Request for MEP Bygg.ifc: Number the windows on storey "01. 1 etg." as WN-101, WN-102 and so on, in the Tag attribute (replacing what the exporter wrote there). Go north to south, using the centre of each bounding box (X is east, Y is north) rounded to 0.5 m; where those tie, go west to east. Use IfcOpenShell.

First a look at what the model holds.

```python
import ifcopenshell
import ifcopenshell.util.element
import ifcopenshell.util.placement

model = ifcopenshell.open("MEP Bygg.ifc")
print(model.schema)
storey = next(s for s in model.by_type("IfcBuildingStorey") if s.Name == "01. 1 etg.")
windows = [e for e in ifcopenshell.util.element.get_decomposition(storey) if e.is_a("IfcWindow")]
for e in sorted(windows, key=lambda e: e.id()):
    origin = ifcopenshell.util.placement.get_local_placement(e.ObjectPlacement)[:3, 3]
    print(e.id(), e.Tag, e.Name, origin.round(2) + 0.0, sep=" | ")
```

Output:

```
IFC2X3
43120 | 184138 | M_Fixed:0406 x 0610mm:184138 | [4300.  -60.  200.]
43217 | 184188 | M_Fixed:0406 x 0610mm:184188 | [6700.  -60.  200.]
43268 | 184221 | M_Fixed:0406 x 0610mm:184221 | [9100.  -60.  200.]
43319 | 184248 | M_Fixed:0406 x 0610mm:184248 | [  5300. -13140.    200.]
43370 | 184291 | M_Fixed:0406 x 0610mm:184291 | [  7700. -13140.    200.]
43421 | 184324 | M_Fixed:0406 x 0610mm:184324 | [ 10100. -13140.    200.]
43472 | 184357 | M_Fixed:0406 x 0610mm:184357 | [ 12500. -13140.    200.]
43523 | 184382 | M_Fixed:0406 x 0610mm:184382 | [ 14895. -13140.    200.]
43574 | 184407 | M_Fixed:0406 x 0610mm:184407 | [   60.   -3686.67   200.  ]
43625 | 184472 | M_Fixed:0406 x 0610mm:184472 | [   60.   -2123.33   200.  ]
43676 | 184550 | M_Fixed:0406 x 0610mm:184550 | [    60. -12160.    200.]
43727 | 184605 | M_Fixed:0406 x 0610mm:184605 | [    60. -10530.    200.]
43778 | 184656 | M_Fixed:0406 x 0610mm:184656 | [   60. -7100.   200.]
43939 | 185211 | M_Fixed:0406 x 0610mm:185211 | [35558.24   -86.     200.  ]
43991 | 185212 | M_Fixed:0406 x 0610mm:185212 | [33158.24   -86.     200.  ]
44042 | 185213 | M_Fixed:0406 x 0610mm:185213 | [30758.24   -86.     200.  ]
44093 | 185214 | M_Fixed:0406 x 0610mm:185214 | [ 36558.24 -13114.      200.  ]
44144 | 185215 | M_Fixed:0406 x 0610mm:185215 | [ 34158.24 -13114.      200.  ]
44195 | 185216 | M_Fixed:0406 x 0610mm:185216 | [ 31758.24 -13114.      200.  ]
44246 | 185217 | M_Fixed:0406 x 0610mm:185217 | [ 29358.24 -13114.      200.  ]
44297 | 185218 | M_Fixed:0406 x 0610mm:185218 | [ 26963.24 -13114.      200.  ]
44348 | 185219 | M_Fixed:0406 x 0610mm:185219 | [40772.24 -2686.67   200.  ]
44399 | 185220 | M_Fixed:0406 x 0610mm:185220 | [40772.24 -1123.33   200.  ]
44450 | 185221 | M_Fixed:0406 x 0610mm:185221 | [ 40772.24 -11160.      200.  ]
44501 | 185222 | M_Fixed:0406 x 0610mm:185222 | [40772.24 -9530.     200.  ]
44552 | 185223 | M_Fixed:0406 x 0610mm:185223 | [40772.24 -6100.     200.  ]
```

```python
import ifcopenshell
import ifcopenshell.geom
import ifcopenshell.util.element
import ifcopenshell.util.shape

model = ifcopenshell.open("MEP Bygg.ifc")
settings = ifcopenshell.geom.settings()
settings.set("use-world-coords", True)


def centre(element):
    shape = ifcopenshell.geom.create_shape(settings, element)
    return ifcopenshell.util.shape.get_bbox_centroid(shape.geometry)


storey = next(s for s in model.by_type("IfcBuildingStorey") if s.Name == "01. 1 etg.")
windows = [e for e in ifcopenshell.util.element.get_decomposition(storey) if e.is_a("IfcWindow")]

# Insertion points can sit at a corner or the storey origin, so sort by the geometry (in metres).
centres = {e: centre(e) for e in windows}
windows.sort(key=lambda e: (-round(centres[e][1] / 0.5), centres[e][0]))

for i, e in enumerate(windows, start=1):
    number = f"WN-1{i:02d}"
    e.Tag = number
    print(e.id(), number)

model.write("MEP Bygg_v2.ifc")
```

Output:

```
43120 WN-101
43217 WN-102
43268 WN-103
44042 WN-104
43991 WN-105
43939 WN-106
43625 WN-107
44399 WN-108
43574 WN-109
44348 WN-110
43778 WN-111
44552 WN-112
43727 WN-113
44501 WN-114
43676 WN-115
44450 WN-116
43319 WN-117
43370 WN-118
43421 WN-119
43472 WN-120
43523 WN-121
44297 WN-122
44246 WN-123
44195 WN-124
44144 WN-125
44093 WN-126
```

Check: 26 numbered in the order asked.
